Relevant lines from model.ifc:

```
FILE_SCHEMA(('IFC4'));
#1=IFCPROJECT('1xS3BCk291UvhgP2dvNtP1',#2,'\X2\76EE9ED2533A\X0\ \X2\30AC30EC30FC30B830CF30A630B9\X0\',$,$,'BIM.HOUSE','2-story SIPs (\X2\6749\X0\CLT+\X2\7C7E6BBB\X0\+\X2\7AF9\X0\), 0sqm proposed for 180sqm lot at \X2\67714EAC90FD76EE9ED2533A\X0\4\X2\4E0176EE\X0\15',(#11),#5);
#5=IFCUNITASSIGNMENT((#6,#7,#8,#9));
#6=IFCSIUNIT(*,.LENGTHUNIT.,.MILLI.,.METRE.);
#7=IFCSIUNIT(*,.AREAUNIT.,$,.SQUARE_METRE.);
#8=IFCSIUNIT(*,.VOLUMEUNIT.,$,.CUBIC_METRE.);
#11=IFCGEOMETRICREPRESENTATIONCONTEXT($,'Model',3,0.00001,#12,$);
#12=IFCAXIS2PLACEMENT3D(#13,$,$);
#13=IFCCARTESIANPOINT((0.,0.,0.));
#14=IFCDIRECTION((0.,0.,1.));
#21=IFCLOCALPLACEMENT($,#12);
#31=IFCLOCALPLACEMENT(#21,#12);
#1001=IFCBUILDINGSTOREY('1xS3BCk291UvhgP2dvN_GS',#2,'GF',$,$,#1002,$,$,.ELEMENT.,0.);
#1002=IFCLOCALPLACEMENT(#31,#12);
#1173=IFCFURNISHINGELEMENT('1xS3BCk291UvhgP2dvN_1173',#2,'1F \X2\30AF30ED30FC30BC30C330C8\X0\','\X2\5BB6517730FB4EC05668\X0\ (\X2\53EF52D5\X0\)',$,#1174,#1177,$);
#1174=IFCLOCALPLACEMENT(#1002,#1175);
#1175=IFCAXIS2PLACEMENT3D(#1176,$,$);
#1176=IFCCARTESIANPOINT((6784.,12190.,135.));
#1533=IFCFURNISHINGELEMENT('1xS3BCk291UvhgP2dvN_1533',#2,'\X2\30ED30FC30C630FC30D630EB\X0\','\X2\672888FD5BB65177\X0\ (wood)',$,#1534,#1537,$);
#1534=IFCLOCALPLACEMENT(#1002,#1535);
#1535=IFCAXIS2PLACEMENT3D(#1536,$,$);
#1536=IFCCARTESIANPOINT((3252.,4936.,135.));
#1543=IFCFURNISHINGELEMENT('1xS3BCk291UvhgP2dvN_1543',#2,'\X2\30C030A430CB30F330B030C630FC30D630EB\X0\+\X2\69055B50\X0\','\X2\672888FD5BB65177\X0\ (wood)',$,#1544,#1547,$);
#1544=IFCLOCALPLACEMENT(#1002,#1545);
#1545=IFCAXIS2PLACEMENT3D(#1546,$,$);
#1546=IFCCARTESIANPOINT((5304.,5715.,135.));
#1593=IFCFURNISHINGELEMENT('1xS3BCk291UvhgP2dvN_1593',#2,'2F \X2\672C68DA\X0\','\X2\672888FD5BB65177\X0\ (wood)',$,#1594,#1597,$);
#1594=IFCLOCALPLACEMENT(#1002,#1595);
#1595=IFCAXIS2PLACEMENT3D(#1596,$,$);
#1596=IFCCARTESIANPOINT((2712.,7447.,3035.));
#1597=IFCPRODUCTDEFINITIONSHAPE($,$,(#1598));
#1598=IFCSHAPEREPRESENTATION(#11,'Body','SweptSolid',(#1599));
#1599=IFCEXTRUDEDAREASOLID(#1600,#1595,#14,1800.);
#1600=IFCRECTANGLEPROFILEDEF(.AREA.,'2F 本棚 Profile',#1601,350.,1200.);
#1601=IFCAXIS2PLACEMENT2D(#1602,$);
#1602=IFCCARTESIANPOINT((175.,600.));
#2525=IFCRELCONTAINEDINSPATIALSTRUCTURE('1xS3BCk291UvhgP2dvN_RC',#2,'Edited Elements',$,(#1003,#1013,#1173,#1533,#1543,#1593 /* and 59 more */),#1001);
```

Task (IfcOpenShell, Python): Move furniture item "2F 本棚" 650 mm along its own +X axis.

```python
import ifcopenshell
import ifcopenshell.api.geometry
import ifcopenshell.util.placement
import ifcopenshell.util.unit

model = ifcopenshell.open("model.ifc")
unit_scale = ifcopenshell.util.unit.calculate_unit_scale(model)

item = model.by_id(1593)
matrix = ifcopenshell.util.placement.get_local_placement(item.ObjectPlacement)
matrix[:3, 3] += matrix[:3, 0] * 0.65 / unit_scale
ifcopenshell.api.geometry.edit_object_placement(model, product=item, matrix=matrix, is_si=False)

print(ifcopenshell.util.placement.get_local_placement(item.ObjectPlacement).round(3) + 0.0)

model.write("model_v2.ifc")
```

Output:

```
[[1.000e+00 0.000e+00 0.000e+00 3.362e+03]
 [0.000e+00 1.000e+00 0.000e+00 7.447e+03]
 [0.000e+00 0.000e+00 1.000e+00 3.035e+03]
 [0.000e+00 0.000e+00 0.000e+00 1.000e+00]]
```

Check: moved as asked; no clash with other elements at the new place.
